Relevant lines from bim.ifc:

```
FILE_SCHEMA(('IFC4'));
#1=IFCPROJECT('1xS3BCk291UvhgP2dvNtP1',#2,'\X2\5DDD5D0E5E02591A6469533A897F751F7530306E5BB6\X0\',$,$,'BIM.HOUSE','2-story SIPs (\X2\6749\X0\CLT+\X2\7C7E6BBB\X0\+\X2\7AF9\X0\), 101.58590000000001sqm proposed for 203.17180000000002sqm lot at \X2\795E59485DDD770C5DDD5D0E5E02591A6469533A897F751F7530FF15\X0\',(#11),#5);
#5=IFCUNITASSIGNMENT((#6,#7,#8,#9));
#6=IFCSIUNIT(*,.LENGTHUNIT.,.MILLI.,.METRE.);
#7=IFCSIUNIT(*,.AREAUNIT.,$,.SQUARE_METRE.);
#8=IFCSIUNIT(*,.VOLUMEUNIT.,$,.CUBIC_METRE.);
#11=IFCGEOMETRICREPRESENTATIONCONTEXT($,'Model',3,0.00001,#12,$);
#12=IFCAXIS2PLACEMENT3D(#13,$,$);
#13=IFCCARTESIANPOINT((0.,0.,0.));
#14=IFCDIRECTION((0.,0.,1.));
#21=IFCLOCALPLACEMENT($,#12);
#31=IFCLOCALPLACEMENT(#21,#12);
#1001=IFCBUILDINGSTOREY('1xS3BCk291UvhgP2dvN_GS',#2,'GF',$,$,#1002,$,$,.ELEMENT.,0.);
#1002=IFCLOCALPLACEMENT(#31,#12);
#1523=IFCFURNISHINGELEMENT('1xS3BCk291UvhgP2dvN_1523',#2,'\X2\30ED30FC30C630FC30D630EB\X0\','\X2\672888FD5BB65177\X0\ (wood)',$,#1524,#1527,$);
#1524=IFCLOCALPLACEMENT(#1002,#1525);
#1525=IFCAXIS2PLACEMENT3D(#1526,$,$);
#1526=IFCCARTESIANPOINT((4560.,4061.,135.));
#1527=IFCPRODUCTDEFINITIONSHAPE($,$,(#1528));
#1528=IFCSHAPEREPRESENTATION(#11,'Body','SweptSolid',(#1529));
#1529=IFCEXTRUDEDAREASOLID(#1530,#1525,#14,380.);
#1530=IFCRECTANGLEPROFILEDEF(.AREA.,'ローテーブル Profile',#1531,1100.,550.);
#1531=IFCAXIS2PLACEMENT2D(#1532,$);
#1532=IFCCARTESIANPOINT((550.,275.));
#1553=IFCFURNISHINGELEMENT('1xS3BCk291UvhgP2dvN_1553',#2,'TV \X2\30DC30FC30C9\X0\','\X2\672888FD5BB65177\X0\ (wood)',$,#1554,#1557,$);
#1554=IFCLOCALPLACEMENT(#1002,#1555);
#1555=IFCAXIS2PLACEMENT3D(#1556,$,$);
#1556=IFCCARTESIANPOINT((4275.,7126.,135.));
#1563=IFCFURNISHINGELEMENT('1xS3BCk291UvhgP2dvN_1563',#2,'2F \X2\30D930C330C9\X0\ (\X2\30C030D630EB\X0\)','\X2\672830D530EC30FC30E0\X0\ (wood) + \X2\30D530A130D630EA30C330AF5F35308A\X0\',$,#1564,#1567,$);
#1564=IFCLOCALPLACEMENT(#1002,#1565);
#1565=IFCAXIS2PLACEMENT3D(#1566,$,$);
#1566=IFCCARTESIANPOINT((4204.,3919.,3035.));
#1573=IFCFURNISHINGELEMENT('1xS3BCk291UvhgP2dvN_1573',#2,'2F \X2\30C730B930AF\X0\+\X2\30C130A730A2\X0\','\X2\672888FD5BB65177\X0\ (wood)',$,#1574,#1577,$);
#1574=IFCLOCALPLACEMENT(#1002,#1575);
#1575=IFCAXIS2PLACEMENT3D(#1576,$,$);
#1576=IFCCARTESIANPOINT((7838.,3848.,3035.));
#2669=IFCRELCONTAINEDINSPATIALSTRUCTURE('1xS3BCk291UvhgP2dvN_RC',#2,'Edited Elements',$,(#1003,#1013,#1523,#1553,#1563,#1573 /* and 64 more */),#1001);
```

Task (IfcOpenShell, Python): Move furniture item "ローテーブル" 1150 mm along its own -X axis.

```python
import ifcopenshell
import ifcopenshell.api.geometry
import ifcopenshell.util.placement

model = ifcopenshell.open("bim.ifc")

item = model.by_guid("1xS3BCk291UvhgP2dvN_1523")
matrix = ifcopenshell.util.placement.get_local_placement(item.ObjectPlacement)
matrix[:3, 3] -= matrix[:3, 0] * 1150.0
ifcopenshell.api.geometry.edit_object_placement(model, product=item, matrix=matrix, is_si=False)

print(ifcopenshell.util.placement.get_local_placement(item.ObjectPlacement).round(3) + 0.0)

model.write("bim_v2.ifc")
```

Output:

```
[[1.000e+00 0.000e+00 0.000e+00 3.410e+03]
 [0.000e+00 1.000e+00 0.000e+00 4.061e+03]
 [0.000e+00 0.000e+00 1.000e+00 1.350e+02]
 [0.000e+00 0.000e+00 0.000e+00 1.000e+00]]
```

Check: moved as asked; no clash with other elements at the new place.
